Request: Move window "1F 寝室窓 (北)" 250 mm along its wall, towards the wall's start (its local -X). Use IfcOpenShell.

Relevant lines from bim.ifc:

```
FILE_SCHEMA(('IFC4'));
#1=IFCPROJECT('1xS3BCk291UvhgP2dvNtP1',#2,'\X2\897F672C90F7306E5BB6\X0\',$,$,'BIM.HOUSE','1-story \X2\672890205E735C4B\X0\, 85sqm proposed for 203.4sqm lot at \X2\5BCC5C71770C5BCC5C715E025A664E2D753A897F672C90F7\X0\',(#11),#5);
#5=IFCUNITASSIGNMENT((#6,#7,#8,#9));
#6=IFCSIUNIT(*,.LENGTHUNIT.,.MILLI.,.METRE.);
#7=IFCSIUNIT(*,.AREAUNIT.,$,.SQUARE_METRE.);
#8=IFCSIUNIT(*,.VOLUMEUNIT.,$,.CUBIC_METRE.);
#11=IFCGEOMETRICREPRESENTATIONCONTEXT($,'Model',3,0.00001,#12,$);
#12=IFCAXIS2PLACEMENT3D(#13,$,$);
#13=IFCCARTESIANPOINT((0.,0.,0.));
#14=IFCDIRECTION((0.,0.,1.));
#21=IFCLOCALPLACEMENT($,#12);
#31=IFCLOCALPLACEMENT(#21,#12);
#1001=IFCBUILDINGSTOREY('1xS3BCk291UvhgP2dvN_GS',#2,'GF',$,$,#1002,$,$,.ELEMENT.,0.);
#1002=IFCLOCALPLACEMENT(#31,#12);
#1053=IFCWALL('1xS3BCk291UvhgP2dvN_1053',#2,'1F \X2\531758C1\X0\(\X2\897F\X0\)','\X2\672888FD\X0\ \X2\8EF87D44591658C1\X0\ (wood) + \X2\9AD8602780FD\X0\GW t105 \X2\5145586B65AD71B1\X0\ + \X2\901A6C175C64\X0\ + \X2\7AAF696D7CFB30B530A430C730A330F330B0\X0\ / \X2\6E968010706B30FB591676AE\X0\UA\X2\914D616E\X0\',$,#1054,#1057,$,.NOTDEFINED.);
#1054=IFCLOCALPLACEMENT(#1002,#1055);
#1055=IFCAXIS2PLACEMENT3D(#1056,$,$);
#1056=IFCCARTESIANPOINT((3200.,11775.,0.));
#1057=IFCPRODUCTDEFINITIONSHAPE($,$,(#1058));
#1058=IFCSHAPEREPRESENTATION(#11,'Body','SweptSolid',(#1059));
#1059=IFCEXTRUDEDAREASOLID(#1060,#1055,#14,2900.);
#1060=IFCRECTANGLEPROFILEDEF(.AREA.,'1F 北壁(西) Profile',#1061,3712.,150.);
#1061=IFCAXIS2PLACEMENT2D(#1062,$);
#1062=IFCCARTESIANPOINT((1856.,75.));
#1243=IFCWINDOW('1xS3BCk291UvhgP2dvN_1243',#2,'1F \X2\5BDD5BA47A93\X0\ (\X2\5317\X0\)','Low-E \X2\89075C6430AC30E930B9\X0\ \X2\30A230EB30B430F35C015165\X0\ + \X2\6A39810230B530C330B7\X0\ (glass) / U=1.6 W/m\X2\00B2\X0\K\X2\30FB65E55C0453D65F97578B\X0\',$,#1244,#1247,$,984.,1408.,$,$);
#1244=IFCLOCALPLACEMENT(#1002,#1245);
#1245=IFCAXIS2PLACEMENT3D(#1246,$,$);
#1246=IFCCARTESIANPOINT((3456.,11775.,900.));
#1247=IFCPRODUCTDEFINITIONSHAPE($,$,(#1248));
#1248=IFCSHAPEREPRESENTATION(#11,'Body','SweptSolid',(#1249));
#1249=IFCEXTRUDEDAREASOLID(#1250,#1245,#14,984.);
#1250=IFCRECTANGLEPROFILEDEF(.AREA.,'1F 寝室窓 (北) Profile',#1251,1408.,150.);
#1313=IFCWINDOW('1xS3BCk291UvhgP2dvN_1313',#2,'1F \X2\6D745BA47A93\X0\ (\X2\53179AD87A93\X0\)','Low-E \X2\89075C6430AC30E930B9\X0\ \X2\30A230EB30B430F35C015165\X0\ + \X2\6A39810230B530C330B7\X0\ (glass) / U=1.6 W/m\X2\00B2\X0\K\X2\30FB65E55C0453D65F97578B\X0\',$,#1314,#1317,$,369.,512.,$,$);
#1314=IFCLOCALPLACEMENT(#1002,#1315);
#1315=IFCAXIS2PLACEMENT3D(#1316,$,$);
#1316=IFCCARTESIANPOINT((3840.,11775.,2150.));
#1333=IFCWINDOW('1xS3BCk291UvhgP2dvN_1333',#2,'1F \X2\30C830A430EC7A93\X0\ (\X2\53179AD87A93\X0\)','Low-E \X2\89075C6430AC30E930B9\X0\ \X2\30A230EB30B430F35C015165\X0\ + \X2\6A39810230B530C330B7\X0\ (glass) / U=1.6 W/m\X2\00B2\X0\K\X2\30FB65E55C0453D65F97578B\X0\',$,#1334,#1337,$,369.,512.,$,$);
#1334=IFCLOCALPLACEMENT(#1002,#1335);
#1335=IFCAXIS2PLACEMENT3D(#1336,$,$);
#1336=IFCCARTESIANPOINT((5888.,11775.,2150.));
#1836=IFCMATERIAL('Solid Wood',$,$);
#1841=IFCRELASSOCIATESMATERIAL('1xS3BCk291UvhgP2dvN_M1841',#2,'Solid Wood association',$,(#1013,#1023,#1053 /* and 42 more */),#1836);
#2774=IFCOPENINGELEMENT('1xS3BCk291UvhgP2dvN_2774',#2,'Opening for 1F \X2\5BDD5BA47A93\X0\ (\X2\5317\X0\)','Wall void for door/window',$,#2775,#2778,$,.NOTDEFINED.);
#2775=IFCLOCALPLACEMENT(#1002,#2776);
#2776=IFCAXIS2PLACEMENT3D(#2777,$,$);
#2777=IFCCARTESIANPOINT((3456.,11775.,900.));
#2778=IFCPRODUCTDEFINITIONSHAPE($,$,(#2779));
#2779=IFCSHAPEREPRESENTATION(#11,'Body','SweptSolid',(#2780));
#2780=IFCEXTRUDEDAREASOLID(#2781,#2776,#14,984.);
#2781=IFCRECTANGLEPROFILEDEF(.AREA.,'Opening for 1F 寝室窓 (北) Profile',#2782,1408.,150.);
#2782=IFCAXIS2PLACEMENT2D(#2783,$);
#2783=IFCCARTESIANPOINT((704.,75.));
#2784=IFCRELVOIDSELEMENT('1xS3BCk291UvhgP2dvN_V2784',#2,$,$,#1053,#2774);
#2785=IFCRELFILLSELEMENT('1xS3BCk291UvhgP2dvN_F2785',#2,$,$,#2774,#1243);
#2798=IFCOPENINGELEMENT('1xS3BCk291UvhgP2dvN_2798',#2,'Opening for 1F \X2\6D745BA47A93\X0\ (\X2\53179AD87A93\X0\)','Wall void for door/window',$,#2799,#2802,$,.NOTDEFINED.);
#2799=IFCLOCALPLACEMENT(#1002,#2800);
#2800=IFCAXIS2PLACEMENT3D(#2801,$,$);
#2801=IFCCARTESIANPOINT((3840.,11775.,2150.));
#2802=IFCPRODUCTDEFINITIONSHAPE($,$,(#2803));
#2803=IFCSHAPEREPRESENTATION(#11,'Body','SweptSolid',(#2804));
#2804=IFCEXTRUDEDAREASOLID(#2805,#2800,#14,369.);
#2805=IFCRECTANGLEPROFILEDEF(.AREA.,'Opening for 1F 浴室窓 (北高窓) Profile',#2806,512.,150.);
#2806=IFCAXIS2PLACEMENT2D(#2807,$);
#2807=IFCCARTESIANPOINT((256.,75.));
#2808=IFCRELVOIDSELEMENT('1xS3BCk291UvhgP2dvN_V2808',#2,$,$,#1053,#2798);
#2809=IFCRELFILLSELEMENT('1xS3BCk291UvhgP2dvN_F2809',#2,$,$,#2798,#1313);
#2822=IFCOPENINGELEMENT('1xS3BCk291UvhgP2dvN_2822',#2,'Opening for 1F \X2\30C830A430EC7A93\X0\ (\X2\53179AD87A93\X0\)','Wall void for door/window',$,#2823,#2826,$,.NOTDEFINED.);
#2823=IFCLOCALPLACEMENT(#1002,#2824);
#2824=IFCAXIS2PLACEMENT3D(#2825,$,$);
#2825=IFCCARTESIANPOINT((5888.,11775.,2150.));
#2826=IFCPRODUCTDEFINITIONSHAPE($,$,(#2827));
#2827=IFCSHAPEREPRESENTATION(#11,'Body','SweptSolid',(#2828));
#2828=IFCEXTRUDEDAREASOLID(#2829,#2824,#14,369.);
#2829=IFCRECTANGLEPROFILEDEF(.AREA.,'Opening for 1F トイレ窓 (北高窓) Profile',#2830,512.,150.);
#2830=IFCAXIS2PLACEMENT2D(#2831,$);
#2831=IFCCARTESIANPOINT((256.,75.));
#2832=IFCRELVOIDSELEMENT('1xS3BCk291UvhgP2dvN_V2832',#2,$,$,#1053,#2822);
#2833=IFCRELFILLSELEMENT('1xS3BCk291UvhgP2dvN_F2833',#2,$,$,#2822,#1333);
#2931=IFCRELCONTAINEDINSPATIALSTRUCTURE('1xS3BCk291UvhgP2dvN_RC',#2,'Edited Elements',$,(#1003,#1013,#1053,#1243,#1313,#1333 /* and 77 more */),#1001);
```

```python
import ifcopenshell
import ifcopenshell.api.geometry
import ifcopenshell.util.placement
import ifcopenshell.util.unit

model = ifcopenshell.open("bim.ifc")
unit_scale = ifcopenshell.util.unit.calculate_unit_scale(model)

window = model.by_guid("1xS3BCk291UvhgP2dvN_1243")
opening = window.FillsVoids[0].RelatingOpeningElement
wall = opening.VoidsElements[0].RelatingBuildingElement

wall_matrix = ifcopenshell.util.placement.get_local_placement(wall.ObjectPlacement)
shift = wall_matrix[:3, 0] * -0.25 / unit_scale
before = ifcopenshell.util.placement.get_local_placement(window.ObjectPlacement)[:3, 3].copy()

# The window is not placed relative to its opening, so move both.
for product in (opening, window):
    matrix = ifcopenshell.util.placement.get_local_placement(product.ObjectPlacement)
    matrix[:3, 3] += shift
    ifcopenshell.api.geometry.edit_object_placement(model, product=product, matrix=matrix, is_si=False)

after = ifcopenshell.util.placement.get_local_placement(window.ObjectPlacement)[:3, 3]
print("window moved by", (after - before).round(3) + 0.0)

model.write("bim_edited.ifc")
```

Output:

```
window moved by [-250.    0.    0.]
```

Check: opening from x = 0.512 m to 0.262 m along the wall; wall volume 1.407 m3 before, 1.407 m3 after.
